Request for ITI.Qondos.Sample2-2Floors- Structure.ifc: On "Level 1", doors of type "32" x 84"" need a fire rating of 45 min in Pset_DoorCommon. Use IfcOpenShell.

First a look at what the model holds.

```python
import ifcopenshell
import ifcopenshell.util.element

model = ifcopenshell.open("ITI.Qondos.Sample2-2Floors- Structure.ifc")
print(model.schema)
storey = next(s for s in model.by_type("IfcBuildingStorey") if s.Name == "Level 1")
doors = [e for e in ifcopenshell.util.element.get_decomposition(storey) if e.is_a("IfcDoor")]
seen = {}
for e in doors:
    element_type = ifcopenshell.util.element.get_type(e)
    key = (element_type.Name if element_type != e and element_type else None, ifcopenshell.util.element.get_pset(e, "Pset_DoorCommon", "FireRating"))
    seen[key] = seen.get(key, 0) + 1
for (name, value), count in sorted(seen.items(), key=str):
    print(count, "x", name, "|", value)
```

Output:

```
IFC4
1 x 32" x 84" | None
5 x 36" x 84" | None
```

```python
import ifcopenshell
import ifcopenshell.api.pset
import ifcopenshell.util.element

model = ifcopenshell.open("ITI.Qondos.Sample2-2Floors- Structure.ifc")

storey = next(s for s in model.by_type("IfcBuildingStorey") if s.Name == "Level 1")
doors = [e for e in ifcopenshell.util.element.get_decomposition(storey) if e.is_a("IfcDoor")]

count = 0
for e in doors:
    element_type = ifcopenshell.util.element.get_type(e)
    if element_type in (None, e) or element_type.Name != '32" x 84"':
        continue
    # add_pset returns the element's existing set when there is one.
    pset = ifcopenshell.api.pset.add_pset(model, product=e, name="Pset_DoorCommon")
    ifcopenshell.api.pset.edit_pset(model, pset=pset, properties={"FireRating": "45 min"})
    count += 1

print(count, "doors updated")

model.write("ITI.Qondos.Sample2-2Floors- Structure-out.ifc")
```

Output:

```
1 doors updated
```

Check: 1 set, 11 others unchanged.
